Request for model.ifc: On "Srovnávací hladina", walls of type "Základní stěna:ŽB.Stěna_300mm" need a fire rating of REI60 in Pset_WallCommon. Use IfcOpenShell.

First a look at what the model holds.

```python
import ifcopenshell
import ifcopenshell.util.element

model = ifcopenshell.open("model.ifc")
print(model.schema)
storey = next(s for s in model.by_type("IfcBuildingStorey") if s.Name == "Srovnávací hladina")
walls = [e for e in ifcopenshell.util.element.get_decomposition(storey) if e.is_a("IfcWall")]
seen = {}
for e in walls:
    element_type = ifcopenshell.util.element.get_type(e)
    key = (element_type.Name if element_type != e and element_type else None, ifcopenshell.util.element.get_pset(e, "Pset_WallCommon", "FireRating"))
    seen[key] = seen.get(key, 0) + 1
for (name, value), count in sorted(seen.items(), key=str):
    print(count, "x", name, "|", value)
```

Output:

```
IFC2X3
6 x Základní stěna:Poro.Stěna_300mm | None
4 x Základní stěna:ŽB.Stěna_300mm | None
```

```python
import ifcopenshell
import ifcopenshell.api.pset
import ifcopenshell.util.element

model = ifcopenshell.open("model.ifc")

storey = next(s for s in model.by_type("IfcBuildingStorey") if s.Name == "Srovnávací hladina")
walls = [e for e in ifcopenshell.util.element.get_decomposition(storey) if e.is_a("IfcWall")]

count = 0
for e in walls:
    element_type = ifcopenshell.util.element.get_type(e)
    if element_type in (None, e) or element_type.Name != "Základní stěna:ŽB.Stěna_300mm":
        continue
    # add_pset returns the element's existing set when there is one.
    pset = ifcopenshell.api.pset.add_pset(model, product=e, name="Pset_WallCommon")
    ifcopenshell.api.pset.edit_pset(model, pset=pset, properties={"FireRating": "REI60"})
    count += 1

print(count, "walls updated")

model.write("model-out.ifc")
```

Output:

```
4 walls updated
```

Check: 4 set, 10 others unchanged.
